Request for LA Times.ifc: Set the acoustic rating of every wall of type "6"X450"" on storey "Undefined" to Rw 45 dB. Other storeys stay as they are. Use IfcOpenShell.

First a look at what the model holds.

```python
import ifcopenshell
import ifcopenshell.util.element

model = ifcopenshell.open("LA Times.ifc")
print(model.schema)
storey = next(s for s in model.by_type("IfcBuildingStorey") if s.Name == "Undefined")
walls = [e for e in ifcopenshell.util.element.get_decomposition(storey) if e.is_a("IfcWall")]
seen = {}
for e in walls:
    element_type = ifcopenshell.util.element.get_type(e)
    key = (element_type.Name if element_type != e and element_type else None, ifcopenshell.util.element.get_pset(e, "Pset_WallCommon", "AcousticRating"))
    seen[key] = seen.get(key, 0) + 1
for (name, value), count in sorted(seen.items(), key=str):
    print(count, "x", name, "|", value)
```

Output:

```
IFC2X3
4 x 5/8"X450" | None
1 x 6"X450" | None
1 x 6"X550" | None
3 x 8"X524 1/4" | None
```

```python
import ifcopenshell
import ifcopenshell.api.pset
import ifcopenshell.util.element

model = ifcopenshell.open("LA Times.ifc")

storey = next(s for s in model.by_type("IfcBuildingStorey") if s.Name == "Undefined")
walls = [e for e in ifcopenshell.util.element.get_decomposition(storey) if e.is_a("IfcWall")]

count = 0
for e in walls:
    element_type = ifcopenshell.util.element.get_type(e)
    if element_type in (None, e) or element_type.Name != '6"X450"':
        continue
    # add_pset returns the element's existing set when there is one.
    pset = ifcopenshell.api.pset.add_pset(model, product=e, name="Pset_WallCommon")
    ifcopenshell.api.pset.edit_pset(model, pset=pset, properties={"AcousticRating": "Rw 45 dB"})
    count += 1

print(count, "walls updated")

model.write("LA Times_edited.ifc")
```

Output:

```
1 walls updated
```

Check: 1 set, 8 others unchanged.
